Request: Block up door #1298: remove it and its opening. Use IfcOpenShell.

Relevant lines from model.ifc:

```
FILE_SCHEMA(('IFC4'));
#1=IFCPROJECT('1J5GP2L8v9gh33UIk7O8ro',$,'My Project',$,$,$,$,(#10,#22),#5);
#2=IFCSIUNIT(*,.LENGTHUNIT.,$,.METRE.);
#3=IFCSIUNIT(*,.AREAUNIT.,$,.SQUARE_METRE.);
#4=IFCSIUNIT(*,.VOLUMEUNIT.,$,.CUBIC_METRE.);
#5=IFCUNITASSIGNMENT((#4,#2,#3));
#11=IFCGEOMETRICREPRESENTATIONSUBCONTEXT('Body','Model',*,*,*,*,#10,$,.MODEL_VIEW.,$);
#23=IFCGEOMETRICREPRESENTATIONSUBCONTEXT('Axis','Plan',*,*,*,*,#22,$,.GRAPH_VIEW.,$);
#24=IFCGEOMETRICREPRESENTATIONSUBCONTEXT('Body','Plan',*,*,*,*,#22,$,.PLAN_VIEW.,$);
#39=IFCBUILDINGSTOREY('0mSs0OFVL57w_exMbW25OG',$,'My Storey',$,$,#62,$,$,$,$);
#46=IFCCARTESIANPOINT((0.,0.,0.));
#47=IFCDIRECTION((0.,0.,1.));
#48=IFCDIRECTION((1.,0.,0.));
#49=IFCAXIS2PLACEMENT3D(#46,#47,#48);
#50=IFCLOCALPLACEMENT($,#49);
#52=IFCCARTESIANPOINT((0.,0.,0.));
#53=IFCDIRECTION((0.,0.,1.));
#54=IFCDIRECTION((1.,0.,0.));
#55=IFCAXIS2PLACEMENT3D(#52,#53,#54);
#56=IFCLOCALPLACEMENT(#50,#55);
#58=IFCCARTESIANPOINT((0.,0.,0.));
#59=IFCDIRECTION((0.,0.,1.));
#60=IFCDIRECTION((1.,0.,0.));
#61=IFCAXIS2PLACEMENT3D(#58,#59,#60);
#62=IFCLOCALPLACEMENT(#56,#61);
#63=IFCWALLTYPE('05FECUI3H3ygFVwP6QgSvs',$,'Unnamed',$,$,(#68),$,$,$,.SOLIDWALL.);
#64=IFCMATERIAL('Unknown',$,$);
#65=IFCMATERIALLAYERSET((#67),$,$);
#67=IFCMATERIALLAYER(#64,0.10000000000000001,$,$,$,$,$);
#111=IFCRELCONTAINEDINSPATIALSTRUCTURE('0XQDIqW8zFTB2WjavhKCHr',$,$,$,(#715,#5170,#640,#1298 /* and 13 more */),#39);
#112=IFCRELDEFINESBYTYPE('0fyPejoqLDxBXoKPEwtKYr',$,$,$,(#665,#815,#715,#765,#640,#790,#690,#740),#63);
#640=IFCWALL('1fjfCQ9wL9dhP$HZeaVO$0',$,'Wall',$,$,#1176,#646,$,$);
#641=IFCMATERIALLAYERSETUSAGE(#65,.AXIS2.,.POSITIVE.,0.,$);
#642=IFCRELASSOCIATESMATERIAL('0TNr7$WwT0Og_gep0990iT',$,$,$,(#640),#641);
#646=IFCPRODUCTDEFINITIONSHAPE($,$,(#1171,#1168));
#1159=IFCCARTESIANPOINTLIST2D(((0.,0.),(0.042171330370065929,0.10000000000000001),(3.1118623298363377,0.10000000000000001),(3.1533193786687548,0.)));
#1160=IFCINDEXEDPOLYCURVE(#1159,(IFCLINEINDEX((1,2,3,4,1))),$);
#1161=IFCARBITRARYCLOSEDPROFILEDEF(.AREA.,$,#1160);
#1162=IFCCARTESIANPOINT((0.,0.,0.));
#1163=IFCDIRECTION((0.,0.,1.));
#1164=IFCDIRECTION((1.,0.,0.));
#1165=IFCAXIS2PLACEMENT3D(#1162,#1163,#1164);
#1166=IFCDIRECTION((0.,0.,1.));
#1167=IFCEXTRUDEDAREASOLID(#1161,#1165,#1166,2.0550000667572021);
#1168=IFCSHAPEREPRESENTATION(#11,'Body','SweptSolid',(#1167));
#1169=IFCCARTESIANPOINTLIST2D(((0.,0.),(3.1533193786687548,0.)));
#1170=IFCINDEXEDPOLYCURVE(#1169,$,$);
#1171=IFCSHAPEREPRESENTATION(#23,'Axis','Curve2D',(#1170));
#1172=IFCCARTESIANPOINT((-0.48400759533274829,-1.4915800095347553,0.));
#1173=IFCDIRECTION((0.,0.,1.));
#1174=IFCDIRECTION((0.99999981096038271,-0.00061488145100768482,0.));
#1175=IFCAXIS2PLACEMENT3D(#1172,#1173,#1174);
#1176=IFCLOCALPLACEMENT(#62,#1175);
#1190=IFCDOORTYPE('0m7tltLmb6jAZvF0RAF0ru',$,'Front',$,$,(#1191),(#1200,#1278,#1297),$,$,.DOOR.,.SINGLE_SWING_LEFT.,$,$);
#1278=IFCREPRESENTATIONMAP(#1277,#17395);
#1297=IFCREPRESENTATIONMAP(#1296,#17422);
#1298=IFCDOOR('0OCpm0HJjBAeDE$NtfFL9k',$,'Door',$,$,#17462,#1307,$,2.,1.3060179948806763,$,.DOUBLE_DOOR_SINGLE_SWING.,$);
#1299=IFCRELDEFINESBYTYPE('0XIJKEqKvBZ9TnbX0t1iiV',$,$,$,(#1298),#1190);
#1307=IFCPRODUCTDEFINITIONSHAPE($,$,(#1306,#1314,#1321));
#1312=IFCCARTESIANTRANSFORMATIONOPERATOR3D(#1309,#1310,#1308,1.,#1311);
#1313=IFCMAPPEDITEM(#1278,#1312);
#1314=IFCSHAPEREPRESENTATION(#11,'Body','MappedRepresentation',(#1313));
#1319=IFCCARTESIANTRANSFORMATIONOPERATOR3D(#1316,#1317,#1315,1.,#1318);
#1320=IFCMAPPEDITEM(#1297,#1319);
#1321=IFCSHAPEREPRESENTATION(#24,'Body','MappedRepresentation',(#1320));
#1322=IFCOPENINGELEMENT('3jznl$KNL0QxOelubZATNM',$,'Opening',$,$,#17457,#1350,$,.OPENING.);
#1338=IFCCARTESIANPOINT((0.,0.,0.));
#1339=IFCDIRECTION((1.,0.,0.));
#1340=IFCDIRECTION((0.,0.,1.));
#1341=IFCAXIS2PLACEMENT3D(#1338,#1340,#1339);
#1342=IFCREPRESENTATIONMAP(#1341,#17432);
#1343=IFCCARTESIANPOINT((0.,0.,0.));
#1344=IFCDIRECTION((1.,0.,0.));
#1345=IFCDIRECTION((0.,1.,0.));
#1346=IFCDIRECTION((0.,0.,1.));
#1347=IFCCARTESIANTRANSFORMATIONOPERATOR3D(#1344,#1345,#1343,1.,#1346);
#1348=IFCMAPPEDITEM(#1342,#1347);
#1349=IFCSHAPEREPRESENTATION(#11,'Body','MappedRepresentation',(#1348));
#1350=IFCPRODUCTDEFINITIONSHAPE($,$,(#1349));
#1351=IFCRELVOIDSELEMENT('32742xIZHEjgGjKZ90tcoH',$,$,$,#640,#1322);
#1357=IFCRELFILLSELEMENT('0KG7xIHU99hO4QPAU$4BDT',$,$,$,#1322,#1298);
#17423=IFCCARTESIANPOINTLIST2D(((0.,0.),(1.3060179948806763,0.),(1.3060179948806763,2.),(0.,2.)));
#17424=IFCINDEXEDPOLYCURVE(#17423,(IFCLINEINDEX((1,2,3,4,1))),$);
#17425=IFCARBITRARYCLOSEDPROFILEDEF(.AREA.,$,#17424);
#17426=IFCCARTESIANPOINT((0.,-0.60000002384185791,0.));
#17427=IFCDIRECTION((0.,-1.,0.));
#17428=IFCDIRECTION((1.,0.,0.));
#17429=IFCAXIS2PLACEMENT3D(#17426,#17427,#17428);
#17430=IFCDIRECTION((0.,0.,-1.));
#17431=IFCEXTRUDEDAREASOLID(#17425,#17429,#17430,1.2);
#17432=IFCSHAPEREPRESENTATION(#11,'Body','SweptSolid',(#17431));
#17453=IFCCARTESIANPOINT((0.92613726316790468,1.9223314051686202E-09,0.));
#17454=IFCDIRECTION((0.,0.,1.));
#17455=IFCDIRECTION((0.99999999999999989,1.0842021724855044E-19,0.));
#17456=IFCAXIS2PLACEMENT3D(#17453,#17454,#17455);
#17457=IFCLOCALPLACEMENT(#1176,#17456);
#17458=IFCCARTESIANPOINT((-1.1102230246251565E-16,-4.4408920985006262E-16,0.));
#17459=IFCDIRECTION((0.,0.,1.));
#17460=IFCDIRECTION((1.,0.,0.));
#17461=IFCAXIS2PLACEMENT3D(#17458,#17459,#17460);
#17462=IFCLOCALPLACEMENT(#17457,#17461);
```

```python
import ifcopenshell
import ifcopenshell.api.feature
import ifcopenshell.api.root
import ifcopenshell.geom
import ifcopenshell.util.shape

model = ifcopenshell.open("model.ifc")
settings = ifcopenshell.geom.settings()


def volume(element):
    """Net volume in cubic metres, openings subtracted."""
    shape = ifcopenshell.geom.create_shape(settings, element)
    return ifcopenshell.util.shape.get_volume(shape.geometry)


door = model.by_guid("0OCpm0HJjBAeDE$NtfFL9k")
opening = door.FillsVoids[0].RelatingOpeningElement
wall = opening.VoidsElements[0].RelatingBuildingElement
before = volume(wall)

ifcopenshell.api.root.remove_product(model, product=door)
ifcopenshell.api.feature.remove_feature(model, feature=opening)

after = volume(wall)

print(f"wall volume {before:.3f} -> {after:.3f} m3")

model.write("model_updated.ifc")
```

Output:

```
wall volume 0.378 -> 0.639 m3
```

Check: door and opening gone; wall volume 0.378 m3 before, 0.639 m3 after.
